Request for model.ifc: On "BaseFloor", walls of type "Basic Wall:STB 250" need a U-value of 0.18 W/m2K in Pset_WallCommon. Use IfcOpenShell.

First a look at what the model holds.

```python
import ifcopenshell
import ifcopenshell.util.element

model = ifcopenshell.open("model.ifc")
print(model.schema)
storey = next(s for s in model.by_type("IfcBuildingStorey") if s.Name == "BaseFloor")
walls = [e for e in ifcopenshell.util.element.get_decomposition(storey) if e.is_a("IfcWall")]
seen = {}
for e in walls:
    element_type = ifcopenshell.util.element.get_type(e)
    key = (element_type.Name if element_type != e and element_type else None, ifcopenshell.util.element.get_pset(e, "Pset_WallCommon", "ThermalTransmittance"))
    seen[key] = seen.get(key, 0) + 1
for (name, value), count in sorted(seen.items(), key=str):
    print(count, "x", name, "|", value)
```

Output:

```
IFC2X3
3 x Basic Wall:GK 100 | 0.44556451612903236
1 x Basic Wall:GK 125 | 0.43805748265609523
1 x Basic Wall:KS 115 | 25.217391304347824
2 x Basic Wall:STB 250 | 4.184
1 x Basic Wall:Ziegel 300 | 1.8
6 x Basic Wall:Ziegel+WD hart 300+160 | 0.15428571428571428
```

```python
import ifcopenshell
import ifcopenshell.api.pset
import ifcopenshell.util.element

model = ifcopenshell.open("model.ifc")

storey = next(s for s in model.by_type("IfcBuildingStorey") if s.Name == "BaseFloor")
walls = [e for e in ifcopenshell.util.element.get_decomposition(storey) if e.is_a("IfcWall")]

count = 0
for e in walls:
    element_type = ifcopenshell.util.element.get_type(e)
    if element_type in (None, e) or element_type.Name != "Basic Wall:STB 250":
        continue
    # add_pset returns the element's existing set when there is one.
    pset = ifcopenshell.api.pset.add_pset(model, product=e, name="Pset_WallCommon")
    ifcopenshell.api.pset.edit_pset(model, pset=pset, properties={"ThermalTransmittance": 0.18})
    count += 1

print(count, "walls updated")

model.write("model_updated.ifc")
```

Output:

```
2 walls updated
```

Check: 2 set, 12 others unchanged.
